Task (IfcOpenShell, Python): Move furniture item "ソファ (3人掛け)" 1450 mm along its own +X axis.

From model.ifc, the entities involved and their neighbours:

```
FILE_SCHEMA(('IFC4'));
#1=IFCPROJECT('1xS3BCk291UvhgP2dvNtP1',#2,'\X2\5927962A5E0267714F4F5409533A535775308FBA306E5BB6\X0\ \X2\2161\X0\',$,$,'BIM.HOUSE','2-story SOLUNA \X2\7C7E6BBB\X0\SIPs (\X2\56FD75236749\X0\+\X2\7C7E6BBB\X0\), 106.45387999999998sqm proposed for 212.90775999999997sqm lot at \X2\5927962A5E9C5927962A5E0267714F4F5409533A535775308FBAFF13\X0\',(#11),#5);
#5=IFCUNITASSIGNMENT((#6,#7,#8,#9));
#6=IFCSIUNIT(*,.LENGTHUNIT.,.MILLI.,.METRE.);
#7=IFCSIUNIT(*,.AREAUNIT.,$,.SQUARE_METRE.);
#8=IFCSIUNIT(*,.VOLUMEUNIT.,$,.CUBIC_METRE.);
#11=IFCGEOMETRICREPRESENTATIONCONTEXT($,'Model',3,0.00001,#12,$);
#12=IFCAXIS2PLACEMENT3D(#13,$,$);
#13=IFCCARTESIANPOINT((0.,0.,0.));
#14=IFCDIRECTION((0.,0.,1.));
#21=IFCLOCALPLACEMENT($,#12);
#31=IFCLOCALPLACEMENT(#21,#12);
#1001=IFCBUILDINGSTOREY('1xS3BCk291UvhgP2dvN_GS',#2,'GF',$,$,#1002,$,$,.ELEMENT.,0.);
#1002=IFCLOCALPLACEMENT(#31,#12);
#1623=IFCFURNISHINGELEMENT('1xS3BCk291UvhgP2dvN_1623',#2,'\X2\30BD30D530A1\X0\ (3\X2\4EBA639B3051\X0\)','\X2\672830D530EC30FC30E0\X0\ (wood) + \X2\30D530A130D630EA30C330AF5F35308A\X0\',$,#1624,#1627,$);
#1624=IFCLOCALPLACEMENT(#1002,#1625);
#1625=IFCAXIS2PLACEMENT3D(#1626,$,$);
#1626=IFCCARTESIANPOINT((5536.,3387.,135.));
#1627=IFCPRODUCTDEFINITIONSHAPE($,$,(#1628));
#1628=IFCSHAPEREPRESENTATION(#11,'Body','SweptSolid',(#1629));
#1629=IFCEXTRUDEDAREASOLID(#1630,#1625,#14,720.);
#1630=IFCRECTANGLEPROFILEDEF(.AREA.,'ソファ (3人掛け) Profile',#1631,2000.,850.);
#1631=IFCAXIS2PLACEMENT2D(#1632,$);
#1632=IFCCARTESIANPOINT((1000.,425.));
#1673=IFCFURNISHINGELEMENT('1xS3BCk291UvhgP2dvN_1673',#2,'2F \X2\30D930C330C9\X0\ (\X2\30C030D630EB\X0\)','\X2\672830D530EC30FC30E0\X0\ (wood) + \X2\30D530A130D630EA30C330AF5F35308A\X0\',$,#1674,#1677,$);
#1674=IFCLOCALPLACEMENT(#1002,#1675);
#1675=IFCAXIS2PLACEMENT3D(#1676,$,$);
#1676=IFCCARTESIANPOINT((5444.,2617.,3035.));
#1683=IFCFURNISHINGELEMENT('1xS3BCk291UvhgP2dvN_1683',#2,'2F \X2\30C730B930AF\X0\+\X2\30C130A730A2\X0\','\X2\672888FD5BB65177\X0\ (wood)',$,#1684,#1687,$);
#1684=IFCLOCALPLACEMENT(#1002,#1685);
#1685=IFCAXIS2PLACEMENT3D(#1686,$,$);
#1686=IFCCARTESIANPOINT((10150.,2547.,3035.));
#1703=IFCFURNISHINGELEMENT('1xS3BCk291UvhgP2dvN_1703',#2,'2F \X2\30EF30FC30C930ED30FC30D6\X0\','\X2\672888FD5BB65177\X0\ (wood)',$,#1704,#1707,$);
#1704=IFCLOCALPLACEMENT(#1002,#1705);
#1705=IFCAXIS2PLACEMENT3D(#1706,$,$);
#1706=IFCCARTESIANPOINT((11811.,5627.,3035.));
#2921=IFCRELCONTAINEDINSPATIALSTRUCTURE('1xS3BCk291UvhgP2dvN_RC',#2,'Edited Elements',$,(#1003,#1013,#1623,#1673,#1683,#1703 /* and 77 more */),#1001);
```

```python
import ifcopenshell
import ifcopenshell.api.geometry
import ifcopenshell.util.placement
import ifcopenshell.util.unit

model = ifcopenshell.open("model.ifc")
unit_scale = ifcopenshell.util.unit.calculate_unit_scale(model)

item = model.by_guid("1xS3BCk291UvhgP2dvN_1623")
matrix = ifcopenshell.util.placement.get_local_placement(item.ObjectPlacement)
matrix[:3, 3] += matrix[:3, 0] * 1.45 / unit_scale
ifcopenshell.api.geometry.edit_object_placement(model, product=item, matrix=matrix, is_si=False)

print(ifcopenshell.util.placement.get_local_placement(item.ObjectPlacement).round(3) + 0.0)

model.write("model_edited.ifc")
```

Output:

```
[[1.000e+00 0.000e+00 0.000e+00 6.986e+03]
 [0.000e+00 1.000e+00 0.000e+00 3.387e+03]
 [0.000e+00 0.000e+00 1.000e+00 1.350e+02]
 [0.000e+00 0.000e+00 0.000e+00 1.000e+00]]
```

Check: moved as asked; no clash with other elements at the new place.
